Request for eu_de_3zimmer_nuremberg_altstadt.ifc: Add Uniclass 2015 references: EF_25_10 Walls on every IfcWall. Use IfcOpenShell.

First a look at what the model holds.

```python
import ifcopenshell

model = ifcopenshell.open("eu_de_3zimmer_nuremberg_altstadt.ifc")
print(model.schema)
print("classifications:", [c.Name for c in model.by_type("IfcClassification")])
for ifc_class in ("IfcDoor", "IfcRoof", "IfcStair", "IfcWall", "IfcWindow"):
    print(ifc_class, len(model.by_type(ifc_class)))
```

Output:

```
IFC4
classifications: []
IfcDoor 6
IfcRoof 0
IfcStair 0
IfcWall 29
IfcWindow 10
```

```python
import ifcopenshell
import ifcopenshell.api.classification

model = ifcopenshell.open("eu_de_3zimmer_nuremberg_altstadt.ifc")

system = ifcopenshell.api.classification.add_classification(model, classification="Uniclass 2015")

codes = {
    "IfcWall": ("EF_25_10", "Walls"),
}
for ifc_class, (code, name) in codes.items():
    products = model.by_type(ifc_class)
    ifcopenshell.api.classification.add_reference(
        model, products=products, classification=system, identification=code, name=name
    )
    print(code, len(products))

model.write("eu_de_3zimmer_nuremberg_altstadt_rev.ifc")
```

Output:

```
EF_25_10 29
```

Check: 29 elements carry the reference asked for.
